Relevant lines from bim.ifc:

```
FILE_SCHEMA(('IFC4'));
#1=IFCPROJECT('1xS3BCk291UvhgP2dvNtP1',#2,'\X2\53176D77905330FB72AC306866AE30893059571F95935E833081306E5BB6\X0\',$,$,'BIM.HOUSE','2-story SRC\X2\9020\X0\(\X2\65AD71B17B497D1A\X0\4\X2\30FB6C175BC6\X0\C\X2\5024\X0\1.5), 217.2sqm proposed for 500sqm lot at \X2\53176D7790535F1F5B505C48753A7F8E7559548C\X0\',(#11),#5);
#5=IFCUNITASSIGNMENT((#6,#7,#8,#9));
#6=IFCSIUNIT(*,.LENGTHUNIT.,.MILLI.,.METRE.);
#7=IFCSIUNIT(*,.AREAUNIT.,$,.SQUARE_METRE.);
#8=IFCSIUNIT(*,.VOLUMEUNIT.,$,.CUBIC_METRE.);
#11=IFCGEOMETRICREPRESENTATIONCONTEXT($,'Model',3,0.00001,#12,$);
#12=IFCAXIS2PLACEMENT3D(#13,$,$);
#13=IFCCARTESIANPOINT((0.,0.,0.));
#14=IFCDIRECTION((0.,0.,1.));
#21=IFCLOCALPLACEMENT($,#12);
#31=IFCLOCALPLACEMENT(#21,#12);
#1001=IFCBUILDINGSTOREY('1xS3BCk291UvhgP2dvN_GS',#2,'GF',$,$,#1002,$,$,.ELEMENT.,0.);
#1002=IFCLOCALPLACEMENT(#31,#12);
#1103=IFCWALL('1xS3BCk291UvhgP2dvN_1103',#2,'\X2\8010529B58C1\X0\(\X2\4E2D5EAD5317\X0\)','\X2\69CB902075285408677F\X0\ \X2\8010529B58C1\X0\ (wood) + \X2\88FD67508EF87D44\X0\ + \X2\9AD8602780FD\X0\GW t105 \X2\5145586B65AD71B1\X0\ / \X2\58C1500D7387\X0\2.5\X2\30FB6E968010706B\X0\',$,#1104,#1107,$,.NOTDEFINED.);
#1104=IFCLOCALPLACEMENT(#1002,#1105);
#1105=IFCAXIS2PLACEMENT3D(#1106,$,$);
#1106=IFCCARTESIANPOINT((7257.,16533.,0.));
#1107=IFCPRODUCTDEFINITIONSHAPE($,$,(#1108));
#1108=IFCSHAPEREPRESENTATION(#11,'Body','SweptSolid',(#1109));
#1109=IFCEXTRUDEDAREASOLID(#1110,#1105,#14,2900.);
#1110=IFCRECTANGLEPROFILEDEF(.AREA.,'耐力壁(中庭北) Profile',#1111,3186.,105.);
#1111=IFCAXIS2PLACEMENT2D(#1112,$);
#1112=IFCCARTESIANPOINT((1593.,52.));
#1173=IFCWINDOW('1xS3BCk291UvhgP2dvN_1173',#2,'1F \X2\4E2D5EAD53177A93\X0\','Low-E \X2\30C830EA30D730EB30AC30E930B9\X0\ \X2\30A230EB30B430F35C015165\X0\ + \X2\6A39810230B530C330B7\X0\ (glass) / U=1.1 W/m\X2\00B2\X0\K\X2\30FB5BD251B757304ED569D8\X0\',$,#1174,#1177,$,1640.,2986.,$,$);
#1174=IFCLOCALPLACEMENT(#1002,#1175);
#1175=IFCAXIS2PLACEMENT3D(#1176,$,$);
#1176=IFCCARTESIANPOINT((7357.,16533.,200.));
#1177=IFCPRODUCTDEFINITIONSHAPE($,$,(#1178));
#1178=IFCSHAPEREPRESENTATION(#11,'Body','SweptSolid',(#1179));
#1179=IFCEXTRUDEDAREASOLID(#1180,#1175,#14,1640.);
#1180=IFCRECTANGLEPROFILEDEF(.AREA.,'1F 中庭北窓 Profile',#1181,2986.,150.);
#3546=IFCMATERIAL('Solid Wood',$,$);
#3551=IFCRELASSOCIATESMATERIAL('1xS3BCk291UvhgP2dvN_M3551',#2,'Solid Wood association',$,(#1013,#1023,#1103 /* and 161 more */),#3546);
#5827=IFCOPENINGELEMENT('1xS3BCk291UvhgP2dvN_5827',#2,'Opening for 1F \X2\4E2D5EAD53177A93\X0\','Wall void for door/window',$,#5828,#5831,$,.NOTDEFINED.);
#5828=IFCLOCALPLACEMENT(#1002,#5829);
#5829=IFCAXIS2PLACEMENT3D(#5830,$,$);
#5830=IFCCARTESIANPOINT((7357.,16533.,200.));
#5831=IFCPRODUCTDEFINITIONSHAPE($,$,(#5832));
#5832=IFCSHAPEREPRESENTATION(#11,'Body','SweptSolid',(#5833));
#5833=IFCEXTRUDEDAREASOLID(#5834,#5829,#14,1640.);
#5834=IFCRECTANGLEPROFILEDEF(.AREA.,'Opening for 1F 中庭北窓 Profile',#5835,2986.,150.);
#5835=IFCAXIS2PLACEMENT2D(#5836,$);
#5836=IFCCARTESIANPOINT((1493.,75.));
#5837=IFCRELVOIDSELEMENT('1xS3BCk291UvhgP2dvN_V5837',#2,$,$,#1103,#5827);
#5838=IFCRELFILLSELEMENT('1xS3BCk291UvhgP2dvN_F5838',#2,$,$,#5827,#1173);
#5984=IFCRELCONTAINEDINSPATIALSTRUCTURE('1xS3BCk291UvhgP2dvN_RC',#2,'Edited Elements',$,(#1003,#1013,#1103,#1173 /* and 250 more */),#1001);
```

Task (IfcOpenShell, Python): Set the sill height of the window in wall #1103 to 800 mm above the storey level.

```python
import numpy as np
import ifcopenshell
import ifcopenshell.api.geometry
import ifcopenshell.geom
import ifcopenshell.util.element
import ifcopenshell.util.placement
import ifcopenshell.util.shape
import ifcopenshell.util.unit

model = ifcopenshell.open("bim.ifc")
unit_scale = ifcopenshell.util.unit.calculate_unit_scale(model)

window = model.by_guid("1xS3BCk291UvhgP2dvN_1173")
opening = window.FillsVoids[0].RelatingOpeningElement
storey = ifcopenshell.util.element.get_container(window, ifc_class="IfcBuildingStorey")
level = ifcopenshell.util.placement.get_local_placement(storey.ObjectPlacement)[2, 3]

# The opening's origin need not be at the sill, so measure its lowest point.
shape = ifcopenshell.geom.create_shape(ifcopenshell.geom.settings(), opening)
bottom = ifcopenshell.util.shape.get_shape_bottom_elevation(shape, shape.geometry) / unit_scale
dz = level + 800.0 - bottom

shift = np.array([0.0, 0.0, dz])
# The window is not placed relative to its opening, so move both.
for product in (opening, window):
    matrix = ifcopenshell.util.placement.get_local_placement(product.ObjectPlacement)
    matrix[:3, 3] += shift
    ifcopenshell.api.geometry.edit_object_placement(model, product=product, matrix=matrix, is_si=False)

print(f"moved by {dz * unit_scale:+.3f} m")

model.write("bim_updated.ifc")
```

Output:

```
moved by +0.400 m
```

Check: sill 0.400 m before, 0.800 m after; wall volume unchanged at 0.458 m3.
